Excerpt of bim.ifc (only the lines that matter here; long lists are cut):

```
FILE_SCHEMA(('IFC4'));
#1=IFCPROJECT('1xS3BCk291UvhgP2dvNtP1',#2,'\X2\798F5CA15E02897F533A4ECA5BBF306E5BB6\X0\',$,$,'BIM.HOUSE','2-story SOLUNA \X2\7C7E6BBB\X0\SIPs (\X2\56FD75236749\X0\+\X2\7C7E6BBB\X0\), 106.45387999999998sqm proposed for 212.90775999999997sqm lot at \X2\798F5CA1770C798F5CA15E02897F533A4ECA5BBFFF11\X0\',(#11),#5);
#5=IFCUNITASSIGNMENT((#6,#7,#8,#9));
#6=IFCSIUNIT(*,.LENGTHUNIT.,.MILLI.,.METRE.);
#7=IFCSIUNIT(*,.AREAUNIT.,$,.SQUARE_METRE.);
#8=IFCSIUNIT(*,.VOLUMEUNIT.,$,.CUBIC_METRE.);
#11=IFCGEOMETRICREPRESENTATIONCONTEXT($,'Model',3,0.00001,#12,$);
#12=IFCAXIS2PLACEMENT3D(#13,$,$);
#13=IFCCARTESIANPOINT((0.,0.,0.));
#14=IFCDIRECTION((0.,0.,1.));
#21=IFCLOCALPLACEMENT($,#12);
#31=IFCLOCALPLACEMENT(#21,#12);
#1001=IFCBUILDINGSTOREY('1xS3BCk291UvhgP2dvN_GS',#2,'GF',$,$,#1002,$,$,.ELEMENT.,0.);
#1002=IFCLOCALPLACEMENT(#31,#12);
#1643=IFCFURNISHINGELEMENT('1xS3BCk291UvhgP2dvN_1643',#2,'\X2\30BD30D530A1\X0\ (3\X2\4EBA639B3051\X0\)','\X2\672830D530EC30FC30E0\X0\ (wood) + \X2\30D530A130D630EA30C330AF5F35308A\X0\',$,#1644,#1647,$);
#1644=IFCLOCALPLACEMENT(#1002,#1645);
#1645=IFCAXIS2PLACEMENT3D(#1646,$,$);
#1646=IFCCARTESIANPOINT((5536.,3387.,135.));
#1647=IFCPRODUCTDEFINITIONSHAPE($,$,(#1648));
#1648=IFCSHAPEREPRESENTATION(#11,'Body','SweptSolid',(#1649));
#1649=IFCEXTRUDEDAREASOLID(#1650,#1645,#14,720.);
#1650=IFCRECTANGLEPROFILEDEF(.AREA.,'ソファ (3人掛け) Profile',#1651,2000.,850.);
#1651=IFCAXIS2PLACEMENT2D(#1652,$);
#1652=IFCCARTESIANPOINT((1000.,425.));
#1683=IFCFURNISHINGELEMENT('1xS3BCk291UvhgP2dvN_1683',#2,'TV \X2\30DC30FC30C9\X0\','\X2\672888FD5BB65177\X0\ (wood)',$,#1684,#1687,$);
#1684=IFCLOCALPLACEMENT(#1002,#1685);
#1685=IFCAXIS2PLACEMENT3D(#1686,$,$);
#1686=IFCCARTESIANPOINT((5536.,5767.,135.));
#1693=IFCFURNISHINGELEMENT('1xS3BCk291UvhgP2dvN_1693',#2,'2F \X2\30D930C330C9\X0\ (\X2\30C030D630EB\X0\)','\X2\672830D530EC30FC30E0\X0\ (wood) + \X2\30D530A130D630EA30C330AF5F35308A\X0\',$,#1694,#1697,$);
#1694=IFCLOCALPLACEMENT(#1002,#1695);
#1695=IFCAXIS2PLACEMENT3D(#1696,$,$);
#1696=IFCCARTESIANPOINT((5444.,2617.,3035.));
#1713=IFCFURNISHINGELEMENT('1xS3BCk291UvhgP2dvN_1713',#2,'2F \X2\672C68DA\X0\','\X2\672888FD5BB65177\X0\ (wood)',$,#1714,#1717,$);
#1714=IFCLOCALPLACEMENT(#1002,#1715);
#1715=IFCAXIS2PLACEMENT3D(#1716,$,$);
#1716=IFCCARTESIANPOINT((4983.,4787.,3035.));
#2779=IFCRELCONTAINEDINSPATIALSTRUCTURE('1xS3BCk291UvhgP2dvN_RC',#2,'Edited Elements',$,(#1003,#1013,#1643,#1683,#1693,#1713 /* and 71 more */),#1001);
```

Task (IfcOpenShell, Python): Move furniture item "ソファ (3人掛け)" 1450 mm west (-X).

```python
import ifcopenshell
import ifcopenshell.api.geometry
import ifcopenshell.util.placement

model = ifcopenshell.open("bim.ifc")

item = model.by_guid("1xS3BCk291UvhgP2dvN_1643")
matrix = ifcopenshell.util.placement.get_local_placement(item.ObjectPlacement)
matrix[0, 3] -= 1450.0
ifcopenshell.api.geometry.edit_object_placement(model, product=item, matrix=matrix, is_si=False)

print(ifcopenshell.util.placement.get_local_placement(item.ObjectPlacement).round(3) + 0.0)

model.write("bim_rev.ifc")
```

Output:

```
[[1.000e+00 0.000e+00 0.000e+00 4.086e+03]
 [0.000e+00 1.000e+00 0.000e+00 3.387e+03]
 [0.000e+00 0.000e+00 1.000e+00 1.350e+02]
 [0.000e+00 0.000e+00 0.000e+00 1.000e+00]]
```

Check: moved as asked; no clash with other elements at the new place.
